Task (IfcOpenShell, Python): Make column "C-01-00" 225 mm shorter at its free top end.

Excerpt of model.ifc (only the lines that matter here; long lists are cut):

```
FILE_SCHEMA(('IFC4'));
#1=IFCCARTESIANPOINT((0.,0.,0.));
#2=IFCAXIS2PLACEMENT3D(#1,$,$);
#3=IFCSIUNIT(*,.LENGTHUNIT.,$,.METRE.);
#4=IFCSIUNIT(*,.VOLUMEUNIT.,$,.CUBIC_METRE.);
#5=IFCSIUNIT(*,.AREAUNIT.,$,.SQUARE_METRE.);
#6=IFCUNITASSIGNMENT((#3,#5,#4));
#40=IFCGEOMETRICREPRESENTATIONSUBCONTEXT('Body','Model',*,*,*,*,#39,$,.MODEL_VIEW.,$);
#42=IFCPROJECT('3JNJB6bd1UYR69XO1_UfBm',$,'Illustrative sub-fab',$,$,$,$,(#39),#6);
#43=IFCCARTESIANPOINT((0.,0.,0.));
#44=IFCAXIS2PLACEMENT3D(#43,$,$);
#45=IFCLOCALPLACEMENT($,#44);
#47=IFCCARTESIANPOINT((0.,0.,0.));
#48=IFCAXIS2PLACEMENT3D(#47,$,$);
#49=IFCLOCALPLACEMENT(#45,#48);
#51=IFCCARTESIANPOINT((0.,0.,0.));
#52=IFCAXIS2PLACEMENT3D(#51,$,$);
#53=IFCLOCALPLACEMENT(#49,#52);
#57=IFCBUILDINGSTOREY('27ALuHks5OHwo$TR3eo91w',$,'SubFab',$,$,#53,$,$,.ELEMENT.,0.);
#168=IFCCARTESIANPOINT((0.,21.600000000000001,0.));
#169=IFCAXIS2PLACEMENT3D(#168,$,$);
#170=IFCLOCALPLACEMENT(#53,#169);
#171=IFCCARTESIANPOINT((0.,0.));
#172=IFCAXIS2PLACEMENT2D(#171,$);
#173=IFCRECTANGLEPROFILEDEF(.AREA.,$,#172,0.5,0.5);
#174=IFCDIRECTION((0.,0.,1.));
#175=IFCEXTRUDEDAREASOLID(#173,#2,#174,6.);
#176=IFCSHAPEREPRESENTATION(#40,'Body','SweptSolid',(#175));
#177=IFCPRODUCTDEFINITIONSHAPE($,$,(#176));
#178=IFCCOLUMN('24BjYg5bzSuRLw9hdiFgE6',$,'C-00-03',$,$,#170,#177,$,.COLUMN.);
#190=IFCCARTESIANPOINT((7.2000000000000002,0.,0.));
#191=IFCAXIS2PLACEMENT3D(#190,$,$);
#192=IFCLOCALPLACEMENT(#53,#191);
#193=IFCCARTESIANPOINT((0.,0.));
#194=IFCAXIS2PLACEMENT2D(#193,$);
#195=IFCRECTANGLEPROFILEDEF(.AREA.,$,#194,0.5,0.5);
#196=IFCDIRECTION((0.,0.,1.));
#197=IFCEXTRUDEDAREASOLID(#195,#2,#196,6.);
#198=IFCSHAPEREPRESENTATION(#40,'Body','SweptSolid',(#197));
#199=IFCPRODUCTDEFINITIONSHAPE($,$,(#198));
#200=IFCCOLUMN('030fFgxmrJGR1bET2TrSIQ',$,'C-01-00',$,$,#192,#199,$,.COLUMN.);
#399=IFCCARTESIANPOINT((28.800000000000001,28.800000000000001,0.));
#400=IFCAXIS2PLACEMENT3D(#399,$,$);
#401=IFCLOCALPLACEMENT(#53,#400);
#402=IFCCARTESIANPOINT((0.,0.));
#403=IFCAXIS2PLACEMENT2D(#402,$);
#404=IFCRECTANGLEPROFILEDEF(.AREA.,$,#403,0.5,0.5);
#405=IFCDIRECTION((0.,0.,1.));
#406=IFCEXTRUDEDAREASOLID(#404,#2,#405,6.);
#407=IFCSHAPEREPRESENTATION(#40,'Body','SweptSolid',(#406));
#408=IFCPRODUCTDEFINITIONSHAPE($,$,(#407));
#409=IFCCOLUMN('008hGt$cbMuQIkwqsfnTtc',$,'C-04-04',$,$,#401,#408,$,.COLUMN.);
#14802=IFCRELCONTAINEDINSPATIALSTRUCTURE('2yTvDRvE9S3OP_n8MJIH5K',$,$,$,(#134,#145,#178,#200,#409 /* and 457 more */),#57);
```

```python
import ifcopenshell
import ifcopenshell.util.representation

model = ifcopenshell.open("model.ifc")

member = model.by_guid("030fFgxmrJGR1bET2TrSIQ")
change = -0.225

# The extrusion runs towards the end named, so only its depth changes.
body = ifcopenshell.util.representation.get_representation(member, "Model", "Body")
solid = body.Items[0]
old_length = solid.Depth
solid.Depth += change

print(f"length {old_length:g} -> {solid.Depth:g}")

model.write("model_edited.ifc")
```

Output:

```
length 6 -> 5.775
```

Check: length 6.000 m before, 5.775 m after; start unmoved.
